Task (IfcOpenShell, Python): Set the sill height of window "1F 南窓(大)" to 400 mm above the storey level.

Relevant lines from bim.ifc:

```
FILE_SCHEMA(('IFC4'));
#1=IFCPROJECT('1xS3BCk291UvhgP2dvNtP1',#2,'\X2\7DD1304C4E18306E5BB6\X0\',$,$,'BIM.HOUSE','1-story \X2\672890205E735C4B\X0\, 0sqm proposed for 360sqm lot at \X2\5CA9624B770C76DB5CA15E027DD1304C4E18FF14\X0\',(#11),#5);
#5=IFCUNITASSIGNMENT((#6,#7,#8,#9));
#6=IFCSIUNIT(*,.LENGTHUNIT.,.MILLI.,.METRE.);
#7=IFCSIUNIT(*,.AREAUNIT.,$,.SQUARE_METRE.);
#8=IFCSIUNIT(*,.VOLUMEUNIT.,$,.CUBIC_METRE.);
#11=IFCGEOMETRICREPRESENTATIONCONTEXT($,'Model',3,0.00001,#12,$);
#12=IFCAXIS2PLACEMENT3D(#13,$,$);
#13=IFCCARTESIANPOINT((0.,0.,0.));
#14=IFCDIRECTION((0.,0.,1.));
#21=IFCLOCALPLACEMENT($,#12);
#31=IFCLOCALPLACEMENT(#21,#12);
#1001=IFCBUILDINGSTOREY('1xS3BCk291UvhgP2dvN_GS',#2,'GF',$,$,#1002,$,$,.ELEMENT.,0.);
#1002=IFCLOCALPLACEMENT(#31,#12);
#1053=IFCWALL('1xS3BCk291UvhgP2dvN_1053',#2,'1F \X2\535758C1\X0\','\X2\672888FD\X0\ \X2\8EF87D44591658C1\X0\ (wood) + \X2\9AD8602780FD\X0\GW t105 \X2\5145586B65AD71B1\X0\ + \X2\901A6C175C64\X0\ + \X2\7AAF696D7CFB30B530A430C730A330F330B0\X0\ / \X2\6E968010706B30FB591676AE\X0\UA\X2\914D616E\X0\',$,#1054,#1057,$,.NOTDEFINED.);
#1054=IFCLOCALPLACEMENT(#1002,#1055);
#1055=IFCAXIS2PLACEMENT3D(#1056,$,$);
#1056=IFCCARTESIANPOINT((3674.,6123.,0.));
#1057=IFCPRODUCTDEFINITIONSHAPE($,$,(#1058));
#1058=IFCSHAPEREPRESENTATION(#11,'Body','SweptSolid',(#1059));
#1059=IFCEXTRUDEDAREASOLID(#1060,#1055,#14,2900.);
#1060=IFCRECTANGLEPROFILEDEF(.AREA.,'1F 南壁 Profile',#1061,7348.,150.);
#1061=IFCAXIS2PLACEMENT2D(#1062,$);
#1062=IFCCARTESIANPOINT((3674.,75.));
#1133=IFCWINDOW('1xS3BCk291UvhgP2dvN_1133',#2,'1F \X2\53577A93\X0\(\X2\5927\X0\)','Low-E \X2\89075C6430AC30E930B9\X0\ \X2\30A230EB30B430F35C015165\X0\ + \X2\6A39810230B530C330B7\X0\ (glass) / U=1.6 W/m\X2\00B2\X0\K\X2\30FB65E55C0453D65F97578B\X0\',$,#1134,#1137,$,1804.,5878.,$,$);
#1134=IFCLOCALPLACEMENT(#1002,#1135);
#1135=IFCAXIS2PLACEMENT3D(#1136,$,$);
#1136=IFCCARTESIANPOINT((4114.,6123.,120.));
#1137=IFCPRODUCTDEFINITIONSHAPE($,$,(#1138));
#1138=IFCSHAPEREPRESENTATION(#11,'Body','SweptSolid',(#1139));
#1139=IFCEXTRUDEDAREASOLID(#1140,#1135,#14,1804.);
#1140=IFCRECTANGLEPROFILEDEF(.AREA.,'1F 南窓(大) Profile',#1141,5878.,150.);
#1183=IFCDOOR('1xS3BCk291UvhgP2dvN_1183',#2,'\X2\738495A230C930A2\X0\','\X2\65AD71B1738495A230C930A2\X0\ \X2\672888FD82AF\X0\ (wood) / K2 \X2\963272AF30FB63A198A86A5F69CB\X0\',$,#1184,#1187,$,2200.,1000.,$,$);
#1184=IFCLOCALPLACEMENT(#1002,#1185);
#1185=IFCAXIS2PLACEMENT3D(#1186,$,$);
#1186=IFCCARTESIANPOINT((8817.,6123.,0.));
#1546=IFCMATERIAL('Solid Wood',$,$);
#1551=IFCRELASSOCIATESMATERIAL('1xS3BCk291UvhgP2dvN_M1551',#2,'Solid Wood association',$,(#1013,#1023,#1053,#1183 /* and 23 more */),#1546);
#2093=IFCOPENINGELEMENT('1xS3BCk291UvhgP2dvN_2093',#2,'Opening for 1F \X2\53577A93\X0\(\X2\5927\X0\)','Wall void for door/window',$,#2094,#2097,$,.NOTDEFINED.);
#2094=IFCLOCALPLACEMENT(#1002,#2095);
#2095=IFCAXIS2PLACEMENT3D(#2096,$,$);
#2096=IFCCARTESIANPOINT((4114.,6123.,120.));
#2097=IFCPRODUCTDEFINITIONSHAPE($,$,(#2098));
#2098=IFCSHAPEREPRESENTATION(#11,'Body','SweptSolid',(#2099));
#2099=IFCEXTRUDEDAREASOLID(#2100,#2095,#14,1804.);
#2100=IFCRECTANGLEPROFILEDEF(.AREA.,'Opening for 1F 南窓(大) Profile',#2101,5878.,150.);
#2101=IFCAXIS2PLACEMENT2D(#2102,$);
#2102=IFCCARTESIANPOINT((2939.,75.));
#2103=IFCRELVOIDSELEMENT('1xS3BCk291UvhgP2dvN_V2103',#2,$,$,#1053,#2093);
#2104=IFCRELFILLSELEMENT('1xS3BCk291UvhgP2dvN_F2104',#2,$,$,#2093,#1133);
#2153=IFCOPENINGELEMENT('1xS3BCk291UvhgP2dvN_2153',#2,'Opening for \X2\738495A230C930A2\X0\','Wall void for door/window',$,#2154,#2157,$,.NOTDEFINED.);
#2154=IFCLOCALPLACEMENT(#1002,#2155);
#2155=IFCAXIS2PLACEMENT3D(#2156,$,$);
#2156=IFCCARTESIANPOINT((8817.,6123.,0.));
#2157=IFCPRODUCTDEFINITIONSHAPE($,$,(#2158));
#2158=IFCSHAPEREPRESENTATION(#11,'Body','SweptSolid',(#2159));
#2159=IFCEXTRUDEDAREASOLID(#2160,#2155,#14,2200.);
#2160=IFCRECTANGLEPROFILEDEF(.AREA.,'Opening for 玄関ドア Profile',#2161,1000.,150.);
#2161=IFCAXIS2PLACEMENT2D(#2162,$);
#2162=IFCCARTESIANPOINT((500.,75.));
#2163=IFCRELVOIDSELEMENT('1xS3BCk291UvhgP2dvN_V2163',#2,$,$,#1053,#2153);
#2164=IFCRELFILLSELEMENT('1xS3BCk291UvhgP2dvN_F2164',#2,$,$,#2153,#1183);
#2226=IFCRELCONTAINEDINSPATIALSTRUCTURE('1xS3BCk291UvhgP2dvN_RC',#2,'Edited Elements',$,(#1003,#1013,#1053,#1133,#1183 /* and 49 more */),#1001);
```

```python
import numpy as np
import ifcopenshell
import ifcopenshell.api.geometry
import ifcopenshell.geom
import ifcopenshell.util.element
import ifcopenshell.util.placement
import ifcopenshell.util.shape
import ifcopenshell.util.unit

model = ifcopenshell.open("bim.ifc")
unit_scale = ifcopenshell.util.unit.calculate_unit_scale(model)

window = model.by_id(1133)
opening = window.FillsVoids[0].RelatingOpeningElement
storey = ifcopenshell.util.element.get_container(window, ifc_class="IfcBuildingStorey")
level = ifcopenshell.util.placement.get_local_placement(storey.ObjectPlacement)[2, 3]

# The opening's origin need not be at the sill, so measure its lowest point.
shape = ifcopenshell.geom.create_shape(ifcopenshell.geom.settings(), opening)
bottom = ifcopenshell.util.shape.get_shape_bottom_elevation(shape, shape.geometry) / unit_scale
dz = level + 400.0 - bottom

shift = np.array([0.0, 0.0, dz])
# The window is not placed relative to its opening, so move both.
for product in (opening, window):
    matrix = ifcopenshell.util.placement.get_local_placement(product.ObjectPlacement)
    matrix[:3, 3] += shift
    ifcopenshell.api.geometry.edit_object_placement(model, product=product, matrix=matrix, is_si=False)

print(f"moved by {dz * unit_scale:+.3f} m")

model.write("bim_rev.ifc")
```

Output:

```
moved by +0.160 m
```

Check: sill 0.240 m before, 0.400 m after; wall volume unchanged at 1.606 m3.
